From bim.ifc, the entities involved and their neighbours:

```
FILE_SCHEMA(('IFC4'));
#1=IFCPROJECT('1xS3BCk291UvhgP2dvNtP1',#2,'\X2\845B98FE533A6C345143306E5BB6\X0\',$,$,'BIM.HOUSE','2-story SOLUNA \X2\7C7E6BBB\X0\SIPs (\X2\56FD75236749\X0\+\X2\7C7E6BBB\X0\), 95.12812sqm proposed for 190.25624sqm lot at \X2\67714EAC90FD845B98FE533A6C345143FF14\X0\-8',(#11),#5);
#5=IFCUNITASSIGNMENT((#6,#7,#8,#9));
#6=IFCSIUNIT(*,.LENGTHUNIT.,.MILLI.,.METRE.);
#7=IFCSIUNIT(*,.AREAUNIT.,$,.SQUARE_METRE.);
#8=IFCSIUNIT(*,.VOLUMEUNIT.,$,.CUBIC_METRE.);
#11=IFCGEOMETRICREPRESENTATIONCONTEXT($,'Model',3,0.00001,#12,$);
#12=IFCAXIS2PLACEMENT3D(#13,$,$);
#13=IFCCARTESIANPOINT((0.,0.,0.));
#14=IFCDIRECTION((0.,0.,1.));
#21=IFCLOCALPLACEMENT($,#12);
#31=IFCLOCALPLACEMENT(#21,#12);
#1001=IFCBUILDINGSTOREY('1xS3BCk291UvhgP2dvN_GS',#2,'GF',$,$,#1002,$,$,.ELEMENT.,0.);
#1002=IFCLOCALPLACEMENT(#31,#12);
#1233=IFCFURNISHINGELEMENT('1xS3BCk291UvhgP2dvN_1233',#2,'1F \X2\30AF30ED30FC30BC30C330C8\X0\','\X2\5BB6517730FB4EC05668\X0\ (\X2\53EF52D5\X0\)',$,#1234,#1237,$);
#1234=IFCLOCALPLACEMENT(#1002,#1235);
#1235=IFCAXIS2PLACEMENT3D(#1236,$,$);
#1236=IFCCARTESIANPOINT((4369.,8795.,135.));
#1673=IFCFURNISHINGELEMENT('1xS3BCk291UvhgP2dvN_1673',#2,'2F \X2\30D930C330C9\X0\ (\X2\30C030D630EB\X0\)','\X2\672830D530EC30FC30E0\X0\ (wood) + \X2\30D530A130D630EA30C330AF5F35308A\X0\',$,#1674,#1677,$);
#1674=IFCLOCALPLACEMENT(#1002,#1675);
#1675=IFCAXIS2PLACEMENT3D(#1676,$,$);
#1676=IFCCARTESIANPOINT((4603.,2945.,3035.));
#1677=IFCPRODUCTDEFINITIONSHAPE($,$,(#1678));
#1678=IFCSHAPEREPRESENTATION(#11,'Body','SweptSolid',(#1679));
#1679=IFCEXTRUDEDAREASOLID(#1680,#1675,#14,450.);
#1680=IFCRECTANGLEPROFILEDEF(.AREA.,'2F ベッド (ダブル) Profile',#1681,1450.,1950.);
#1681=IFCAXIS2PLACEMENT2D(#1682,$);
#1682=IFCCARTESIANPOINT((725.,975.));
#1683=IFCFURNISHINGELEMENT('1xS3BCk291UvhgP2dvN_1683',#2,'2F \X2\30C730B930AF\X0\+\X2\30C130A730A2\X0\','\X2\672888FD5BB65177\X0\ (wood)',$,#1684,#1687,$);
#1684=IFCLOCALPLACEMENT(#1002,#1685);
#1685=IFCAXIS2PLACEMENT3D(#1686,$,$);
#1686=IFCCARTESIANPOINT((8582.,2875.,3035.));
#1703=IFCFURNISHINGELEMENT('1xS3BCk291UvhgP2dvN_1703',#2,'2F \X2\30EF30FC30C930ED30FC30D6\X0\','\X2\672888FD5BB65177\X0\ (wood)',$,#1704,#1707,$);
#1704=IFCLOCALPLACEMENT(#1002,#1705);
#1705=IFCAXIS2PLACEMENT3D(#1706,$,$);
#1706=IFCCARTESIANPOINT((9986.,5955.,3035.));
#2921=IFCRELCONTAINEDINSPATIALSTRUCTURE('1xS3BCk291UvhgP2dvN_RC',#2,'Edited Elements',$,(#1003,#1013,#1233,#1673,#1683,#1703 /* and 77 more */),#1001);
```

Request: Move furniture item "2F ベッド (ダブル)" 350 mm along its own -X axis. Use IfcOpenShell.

```python
import ifcopenshell
import ifcopenshell.api.geometry
import ifcopenshell.util.placement

model = ifcopenshell.open("bim.ifc")

item = model.by_guid("1xS3BCk291UvhgP2dvN_1673")
matrix = ifcopenshell.util.placement.get_local_placement(item.ObjectPlacement)
matrix[:3, 3] -= matrix[:3, 0] * 350.0
ifcopenshell.api.geometry.edit_object_placement(model, product=item, matrix=matrix, is_si=False)

print(ifcopenshell.util.placement.get_local_placement(item.ObjectPlacement).round(3) + 0.0)

model.write("bim_rev.ifc")
```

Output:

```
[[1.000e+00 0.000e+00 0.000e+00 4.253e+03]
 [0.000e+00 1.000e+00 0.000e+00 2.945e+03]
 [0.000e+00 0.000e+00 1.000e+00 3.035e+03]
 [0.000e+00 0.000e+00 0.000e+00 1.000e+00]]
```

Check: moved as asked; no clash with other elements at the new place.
